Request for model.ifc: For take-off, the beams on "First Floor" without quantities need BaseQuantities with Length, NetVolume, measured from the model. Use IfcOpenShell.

First a look at what the model holds.

```python
import ifcopenshell
import ifcopenshell.util.element
import ifcopenshell.util.unit

model = ifcopenshell.open("model.ifc")
print(model.schema)
for unit_type in ("LENGTHUNIT", "AREAUNIT", "VOLUMEUNIT"):
    print(unit_type, ifcopenshell.util.unit.calculate_unit_scale(model, unit_type))
storey = next(s for s in model.by_type("IfcBuildingStorey") if s.Name == "First Floor")
beams = [e for e in ifcopenshell.util.element.get_decomposition(storey) if e.is_a("IfcBeam")]
for e in sorted(beams, key=lambda e: e.id()):
    print(e.id(), e.is_a(), e.Name, list(ifcopenshell.util.element.get_psets(e, qtos_only=True)), sep=" | ")
```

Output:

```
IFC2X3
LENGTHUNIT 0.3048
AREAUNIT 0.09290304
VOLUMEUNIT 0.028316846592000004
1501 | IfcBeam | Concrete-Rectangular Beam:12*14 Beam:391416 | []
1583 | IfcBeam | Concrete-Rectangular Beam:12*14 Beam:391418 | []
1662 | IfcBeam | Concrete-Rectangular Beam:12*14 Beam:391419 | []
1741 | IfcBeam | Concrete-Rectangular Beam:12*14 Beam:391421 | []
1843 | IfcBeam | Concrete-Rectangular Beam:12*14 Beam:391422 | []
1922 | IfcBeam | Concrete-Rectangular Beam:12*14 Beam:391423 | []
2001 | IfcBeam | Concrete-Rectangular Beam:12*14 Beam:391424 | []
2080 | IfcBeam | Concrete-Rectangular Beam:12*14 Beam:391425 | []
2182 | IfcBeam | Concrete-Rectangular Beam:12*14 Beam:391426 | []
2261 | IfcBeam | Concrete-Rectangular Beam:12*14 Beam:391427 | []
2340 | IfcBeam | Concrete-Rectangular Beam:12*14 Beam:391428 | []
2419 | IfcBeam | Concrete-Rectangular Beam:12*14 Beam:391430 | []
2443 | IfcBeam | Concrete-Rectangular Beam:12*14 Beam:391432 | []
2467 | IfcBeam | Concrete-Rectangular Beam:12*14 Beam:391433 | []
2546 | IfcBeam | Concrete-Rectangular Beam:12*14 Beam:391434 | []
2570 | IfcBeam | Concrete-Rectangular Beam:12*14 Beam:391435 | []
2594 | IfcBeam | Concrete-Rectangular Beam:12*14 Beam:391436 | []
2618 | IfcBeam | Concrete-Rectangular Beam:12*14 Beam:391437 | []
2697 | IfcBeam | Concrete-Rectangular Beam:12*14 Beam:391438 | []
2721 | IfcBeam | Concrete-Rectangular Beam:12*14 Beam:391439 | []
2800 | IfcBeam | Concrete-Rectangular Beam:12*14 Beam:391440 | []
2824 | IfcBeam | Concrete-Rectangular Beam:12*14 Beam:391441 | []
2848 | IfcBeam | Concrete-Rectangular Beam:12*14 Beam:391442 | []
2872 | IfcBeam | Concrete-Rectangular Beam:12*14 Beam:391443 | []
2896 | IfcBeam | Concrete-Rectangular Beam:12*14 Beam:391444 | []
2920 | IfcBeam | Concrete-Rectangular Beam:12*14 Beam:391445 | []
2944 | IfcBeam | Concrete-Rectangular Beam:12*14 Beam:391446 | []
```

```python
import ifcopenshell
import ifcopenshell.api.pset
import ifcopenshell.geom
import ifcopenshell.util.element
import ifcopenshell.util.shape
import ifcopenshell.util.unit

model = ifcopenshell.open("model.ifc")
unit_scale = ifcopenshell.util.unit.calculate_unit_scale(model)
volume_scale = ifcopenshell.util.unit.calculate_unit_scale(model, "VOLUMEUNIT")
settings = ifcopenshell.geom.settings()

storey = next(s for s in model.by_type("IfcBuildingStorey") if s.Name == "First Floor")
beams = [e for e in ifcopenshell.util.element.get_decomposition(storey) if e.is_a("IfcBeam")]

for e in sorted(beams, key=lambda e: e.id()):
    if ifcopenshell.util.element.get_psets(e, qtos_only=True, should_inherit=False):
        continue
    # Geometry comes back in metres, in the element's own axes.
    shape = ifcopenshell.geom.create_shape(settings, e)
    values = {
        "Length": ifcopenshell.util.shape.get_max_xyz(shape.geometry) / unit_scale,
        "NetVolume": ifcopenshell.util.shape.get_volume(shape.geometry) / volume_scale,
    }
    qto = ifcopenshell.api.pset.add_qto(model, product=e, name="BaseQuantities")
    ifcopenshell.api.pset.edit_qto(model, qto=qto, properties=values)
    print(e.id(), {k: round(v, 3) for k, v in values.items()})

model.write("model-out.ifc")
```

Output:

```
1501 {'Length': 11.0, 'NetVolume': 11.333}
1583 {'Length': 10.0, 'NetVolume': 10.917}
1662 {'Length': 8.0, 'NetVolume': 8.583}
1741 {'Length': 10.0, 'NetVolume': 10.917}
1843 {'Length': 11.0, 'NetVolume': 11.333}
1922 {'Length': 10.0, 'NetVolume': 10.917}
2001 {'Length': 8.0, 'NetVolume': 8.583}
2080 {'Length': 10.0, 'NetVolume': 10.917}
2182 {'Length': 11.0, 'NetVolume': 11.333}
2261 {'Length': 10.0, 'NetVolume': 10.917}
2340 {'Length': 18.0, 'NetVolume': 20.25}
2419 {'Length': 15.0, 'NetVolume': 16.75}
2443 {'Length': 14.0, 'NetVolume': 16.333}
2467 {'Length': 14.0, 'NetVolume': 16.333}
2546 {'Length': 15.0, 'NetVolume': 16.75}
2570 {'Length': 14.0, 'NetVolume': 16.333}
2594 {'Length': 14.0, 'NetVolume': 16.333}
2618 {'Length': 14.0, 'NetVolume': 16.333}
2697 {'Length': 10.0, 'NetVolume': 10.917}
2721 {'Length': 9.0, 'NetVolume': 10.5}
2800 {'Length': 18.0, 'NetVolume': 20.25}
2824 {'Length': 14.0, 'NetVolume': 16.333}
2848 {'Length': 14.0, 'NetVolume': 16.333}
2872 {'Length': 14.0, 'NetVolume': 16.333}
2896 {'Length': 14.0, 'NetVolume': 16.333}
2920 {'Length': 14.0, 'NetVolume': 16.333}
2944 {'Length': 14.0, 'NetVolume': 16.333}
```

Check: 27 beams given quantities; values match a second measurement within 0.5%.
